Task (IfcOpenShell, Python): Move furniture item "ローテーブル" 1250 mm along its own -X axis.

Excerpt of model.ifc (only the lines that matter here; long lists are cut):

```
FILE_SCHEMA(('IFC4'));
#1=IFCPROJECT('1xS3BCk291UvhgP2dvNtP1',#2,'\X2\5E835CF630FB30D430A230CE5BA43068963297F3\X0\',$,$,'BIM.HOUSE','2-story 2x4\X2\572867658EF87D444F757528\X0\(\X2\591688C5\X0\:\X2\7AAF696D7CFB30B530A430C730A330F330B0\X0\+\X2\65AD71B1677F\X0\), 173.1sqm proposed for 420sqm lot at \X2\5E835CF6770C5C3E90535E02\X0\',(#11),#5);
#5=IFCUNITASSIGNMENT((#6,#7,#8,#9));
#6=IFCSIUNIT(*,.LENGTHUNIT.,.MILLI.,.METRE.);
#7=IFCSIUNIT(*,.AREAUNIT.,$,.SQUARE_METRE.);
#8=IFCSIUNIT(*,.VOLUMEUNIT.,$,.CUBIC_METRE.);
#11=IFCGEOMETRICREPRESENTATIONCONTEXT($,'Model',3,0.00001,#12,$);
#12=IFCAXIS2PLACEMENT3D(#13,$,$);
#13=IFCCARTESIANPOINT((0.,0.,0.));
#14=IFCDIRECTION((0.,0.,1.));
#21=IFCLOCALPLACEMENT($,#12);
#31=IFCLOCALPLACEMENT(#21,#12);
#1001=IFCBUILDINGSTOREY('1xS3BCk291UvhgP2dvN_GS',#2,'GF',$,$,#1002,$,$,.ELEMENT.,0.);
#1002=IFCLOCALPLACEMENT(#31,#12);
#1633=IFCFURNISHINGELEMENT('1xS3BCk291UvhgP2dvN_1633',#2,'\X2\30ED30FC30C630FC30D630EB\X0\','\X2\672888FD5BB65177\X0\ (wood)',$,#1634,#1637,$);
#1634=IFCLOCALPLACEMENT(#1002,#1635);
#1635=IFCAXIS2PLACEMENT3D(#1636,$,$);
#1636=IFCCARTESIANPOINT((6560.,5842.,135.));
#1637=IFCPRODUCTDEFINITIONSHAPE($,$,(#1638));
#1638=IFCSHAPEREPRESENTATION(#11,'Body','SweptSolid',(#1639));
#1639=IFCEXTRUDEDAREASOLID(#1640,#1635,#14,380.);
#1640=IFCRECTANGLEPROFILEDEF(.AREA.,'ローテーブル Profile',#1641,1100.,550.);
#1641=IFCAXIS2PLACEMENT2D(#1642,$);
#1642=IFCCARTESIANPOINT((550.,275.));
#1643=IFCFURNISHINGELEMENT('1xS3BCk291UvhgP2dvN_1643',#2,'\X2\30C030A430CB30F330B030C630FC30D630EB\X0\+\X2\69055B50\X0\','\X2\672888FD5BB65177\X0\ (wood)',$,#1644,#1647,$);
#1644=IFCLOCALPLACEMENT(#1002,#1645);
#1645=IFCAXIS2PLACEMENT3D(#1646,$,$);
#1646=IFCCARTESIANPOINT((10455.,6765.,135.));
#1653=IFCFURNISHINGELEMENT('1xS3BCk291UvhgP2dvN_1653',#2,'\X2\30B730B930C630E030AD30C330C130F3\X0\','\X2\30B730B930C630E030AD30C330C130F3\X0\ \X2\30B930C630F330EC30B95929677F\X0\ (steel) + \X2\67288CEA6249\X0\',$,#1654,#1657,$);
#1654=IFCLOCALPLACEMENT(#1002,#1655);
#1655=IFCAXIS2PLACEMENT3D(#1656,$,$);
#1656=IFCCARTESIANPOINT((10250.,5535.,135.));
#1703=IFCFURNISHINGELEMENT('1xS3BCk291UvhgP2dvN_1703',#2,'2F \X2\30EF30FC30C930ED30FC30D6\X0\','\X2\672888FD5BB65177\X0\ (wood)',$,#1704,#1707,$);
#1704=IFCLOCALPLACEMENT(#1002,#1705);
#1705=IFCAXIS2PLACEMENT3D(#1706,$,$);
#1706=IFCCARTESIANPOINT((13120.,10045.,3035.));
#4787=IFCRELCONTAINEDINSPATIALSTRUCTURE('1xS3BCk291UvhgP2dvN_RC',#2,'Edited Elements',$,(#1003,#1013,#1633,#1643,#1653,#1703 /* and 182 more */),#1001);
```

```python
import ifcopenshell
import ifcopenshell.api.geometry
import ifcopenshell.util.placement
import ifcopenshell.util.unit

model = ifcopenshell.open("model.ifc")
unit_scale = ifcopenshell.util.unit.calculate_unit_scale(model)

item = model.by_id(1633)
matrix = ifcopenshell.util.placement.get_local_placement(item.ObjectPlacement)
matrix[:3, 3] -= matrix[:3, 0] * 1.25 / unit_scale
ifcopenshell.api.geometry.edit_object_placement(model, product=item, matrix=matrix, is_si=False)

print(ifcopenshell.util.placement.get_local_placement(item.ObjectPlacement).round(3) + 0.0)

model.write("model-out.ifc")
```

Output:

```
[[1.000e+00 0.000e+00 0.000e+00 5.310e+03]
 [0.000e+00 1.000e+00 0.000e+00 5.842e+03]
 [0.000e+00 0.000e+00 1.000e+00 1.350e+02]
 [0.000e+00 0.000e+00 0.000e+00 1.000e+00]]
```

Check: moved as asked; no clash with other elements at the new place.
